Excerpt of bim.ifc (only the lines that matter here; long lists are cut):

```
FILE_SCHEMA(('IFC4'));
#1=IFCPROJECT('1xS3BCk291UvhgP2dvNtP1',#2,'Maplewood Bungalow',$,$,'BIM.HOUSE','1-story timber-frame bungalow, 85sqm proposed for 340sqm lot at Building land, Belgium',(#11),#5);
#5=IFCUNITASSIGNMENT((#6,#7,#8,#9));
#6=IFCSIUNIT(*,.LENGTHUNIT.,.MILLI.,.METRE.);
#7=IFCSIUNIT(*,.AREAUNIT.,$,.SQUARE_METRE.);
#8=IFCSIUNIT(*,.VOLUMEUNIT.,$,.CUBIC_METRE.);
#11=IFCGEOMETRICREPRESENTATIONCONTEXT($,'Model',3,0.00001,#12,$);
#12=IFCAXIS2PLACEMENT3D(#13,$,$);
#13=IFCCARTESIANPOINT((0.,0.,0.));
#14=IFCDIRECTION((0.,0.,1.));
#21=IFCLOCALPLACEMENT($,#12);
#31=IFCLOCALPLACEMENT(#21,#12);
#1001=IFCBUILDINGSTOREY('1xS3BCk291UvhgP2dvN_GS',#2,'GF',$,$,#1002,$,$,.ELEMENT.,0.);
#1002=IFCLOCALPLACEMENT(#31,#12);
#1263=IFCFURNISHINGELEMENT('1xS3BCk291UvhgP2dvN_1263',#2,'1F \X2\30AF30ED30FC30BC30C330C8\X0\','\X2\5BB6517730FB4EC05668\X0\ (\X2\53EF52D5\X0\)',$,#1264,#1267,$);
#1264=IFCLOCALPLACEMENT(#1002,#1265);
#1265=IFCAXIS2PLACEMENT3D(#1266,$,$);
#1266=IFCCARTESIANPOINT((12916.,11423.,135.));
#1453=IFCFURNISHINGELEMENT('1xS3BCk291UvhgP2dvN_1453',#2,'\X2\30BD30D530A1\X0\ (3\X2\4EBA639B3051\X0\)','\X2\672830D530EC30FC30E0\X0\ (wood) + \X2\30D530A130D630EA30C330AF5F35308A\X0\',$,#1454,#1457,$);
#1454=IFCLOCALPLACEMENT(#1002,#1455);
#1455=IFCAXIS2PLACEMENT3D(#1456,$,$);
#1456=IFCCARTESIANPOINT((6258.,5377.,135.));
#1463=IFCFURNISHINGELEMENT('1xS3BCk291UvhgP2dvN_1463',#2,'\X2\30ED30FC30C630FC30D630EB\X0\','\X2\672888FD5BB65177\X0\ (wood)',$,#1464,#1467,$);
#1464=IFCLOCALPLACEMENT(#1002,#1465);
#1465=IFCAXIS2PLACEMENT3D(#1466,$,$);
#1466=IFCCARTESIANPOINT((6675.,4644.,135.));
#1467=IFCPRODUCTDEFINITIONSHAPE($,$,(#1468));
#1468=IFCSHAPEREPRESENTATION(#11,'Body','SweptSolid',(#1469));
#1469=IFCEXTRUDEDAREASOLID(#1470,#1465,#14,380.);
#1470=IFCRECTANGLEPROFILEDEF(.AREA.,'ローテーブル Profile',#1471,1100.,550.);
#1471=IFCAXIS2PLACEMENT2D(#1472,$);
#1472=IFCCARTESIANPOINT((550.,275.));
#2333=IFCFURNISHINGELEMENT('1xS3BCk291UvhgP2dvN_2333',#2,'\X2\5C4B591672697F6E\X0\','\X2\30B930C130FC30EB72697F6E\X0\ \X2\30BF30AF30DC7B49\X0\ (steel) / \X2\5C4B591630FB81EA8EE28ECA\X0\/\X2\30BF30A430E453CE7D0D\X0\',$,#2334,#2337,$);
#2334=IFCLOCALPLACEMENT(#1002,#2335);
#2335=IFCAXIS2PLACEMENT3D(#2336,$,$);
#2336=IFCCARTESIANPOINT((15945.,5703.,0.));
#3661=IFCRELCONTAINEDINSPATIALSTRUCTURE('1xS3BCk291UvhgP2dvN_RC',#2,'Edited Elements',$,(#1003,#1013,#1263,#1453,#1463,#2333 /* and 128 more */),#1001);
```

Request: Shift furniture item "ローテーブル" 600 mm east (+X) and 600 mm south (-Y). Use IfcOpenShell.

```python
import ifcopenshell
import ifcopenshell.api.geometry
import ifcopenshell.util.placement

model = ifcopenshell.open("bim.ifc")

item = model.by_guid("1xS3BCk291UvhgP2dvN_1463")
matrix = ifcopenshell.util.placement.get_local_placement(item.ObjectPlacement)
matrix[0, 3] += 600.0
matrix[1, 3] -= 600.0
ifcopenshell.api.geometry.edit_object_placement(model, product=item, matrix=matrix, is_si=False)

print(ifcopenshell.util.placement.get_local_placement(item.ObjectPlacement).round(3) + 0.0)

model.write("bim_edited.ifc")
```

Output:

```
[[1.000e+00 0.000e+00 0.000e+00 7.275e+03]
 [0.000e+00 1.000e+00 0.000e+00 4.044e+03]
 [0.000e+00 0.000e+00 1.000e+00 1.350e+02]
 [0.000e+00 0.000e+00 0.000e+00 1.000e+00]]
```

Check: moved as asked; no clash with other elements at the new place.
